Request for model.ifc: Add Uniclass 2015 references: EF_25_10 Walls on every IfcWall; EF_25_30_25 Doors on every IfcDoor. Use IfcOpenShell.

First a look at what the model holds.

```python
import ifcopenshell

model = ifcopenshell.open("model.ifc")
print(model.schema)
print("classifications:", [c.Name for c in model.by_type("IfcClassification")])
for ifc_class in ("IfcDoor", "IfcRoof", "IfcStair", "IfcWall", "IfcWindow"):
    print(ifc_class, len(model.by_type(ifc_class)))
```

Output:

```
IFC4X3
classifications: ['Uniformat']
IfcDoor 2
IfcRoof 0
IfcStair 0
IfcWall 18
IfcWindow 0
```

```python
import ifcopenshell
import ifcopenshell.api.classification

model = ifcopenshell.open("model.ifc")

system = ifcopenshell.api.classification.add_classification(model, classification="Uniclass 2015")

codes = {
    "IfcWall": ("EF_25_10", "Walls"),
    "IfcDoor": ("EF_25_30_25", "Doors"),
}
for ifc_class, (code, name) in codes.items():
    products = model.by_type(ifc_class)
    ifcopenshell.api.classification.add_reference(
        model, products=products, classification=system, identification=code, name=name
    )
    print(code, len(products))

model.write("model_v2.ifc")
```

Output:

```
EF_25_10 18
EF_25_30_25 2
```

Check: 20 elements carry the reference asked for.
